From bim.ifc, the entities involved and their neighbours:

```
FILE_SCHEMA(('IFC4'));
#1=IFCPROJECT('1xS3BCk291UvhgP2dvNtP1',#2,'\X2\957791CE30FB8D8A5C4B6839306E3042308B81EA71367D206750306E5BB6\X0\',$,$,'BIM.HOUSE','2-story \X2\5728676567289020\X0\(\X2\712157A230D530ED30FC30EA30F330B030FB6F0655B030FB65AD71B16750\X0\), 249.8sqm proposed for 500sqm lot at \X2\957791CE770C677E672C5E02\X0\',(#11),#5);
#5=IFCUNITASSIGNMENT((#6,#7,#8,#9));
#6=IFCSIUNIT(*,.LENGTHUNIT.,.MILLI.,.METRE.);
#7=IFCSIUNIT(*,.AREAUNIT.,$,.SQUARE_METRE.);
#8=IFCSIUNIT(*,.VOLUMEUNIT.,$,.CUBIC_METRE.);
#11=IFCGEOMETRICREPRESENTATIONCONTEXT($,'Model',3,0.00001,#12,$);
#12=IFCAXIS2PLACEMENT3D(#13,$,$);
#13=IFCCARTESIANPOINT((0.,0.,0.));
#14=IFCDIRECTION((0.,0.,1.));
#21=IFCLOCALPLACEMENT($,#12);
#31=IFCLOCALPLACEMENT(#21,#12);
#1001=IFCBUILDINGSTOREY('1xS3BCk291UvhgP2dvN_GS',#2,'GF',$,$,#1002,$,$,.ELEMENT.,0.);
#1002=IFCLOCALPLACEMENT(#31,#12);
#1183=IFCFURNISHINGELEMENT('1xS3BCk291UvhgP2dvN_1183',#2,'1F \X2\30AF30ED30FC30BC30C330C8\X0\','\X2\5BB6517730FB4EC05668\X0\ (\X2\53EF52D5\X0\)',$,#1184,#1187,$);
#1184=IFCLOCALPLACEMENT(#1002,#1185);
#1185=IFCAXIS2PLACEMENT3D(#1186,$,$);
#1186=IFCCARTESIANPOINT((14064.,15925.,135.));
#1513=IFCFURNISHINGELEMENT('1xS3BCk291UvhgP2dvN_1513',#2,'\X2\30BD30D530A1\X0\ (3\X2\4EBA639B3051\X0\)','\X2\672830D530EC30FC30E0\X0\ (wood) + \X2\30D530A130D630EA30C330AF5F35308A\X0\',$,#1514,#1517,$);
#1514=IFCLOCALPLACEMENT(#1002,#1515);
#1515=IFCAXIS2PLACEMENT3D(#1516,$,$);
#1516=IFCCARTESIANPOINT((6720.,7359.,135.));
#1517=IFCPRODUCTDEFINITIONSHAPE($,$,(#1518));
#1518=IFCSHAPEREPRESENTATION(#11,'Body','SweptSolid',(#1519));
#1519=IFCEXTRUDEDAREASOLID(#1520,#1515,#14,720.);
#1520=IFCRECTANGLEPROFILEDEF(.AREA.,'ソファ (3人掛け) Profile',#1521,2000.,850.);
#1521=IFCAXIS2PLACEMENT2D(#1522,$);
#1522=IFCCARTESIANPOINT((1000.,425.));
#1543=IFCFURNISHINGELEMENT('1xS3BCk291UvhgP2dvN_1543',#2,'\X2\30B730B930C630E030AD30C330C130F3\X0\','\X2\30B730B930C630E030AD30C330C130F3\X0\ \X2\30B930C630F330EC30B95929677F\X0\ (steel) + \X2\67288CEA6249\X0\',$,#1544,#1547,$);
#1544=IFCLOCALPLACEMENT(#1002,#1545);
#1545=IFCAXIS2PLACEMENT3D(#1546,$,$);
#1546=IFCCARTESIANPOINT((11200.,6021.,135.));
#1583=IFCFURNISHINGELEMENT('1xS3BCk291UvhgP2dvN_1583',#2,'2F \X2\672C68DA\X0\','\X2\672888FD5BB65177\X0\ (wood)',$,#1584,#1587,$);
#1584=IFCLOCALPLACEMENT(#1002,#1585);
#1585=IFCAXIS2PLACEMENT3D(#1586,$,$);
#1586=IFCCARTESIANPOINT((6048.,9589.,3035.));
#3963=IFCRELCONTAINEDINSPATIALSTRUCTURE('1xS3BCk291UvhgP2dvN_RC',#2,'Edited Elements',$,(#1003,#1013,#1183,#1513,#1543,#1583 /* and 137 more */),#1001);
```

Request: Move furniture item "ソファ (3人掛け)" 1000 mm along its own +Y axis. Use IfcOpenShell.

```python
import ifcopenshell
import ifcopenshell.api.geometry
import ifcopenshell.util.placement
import ifcopenshell.util.unit

model = ifcopenshell.open("bim.ifc")
unit_scale = ifcopenshell.util.unit.calculate_unit_scale(model)

item = model.by_id(1513)
matrix = ifcopenshell.util.placement.get_local_placement(item.ObjectPlacement)
matrix[:3, 3] += matrix[:3, 1] * 1 / unit_scale
ifcopenshell.api.geometry.edit_object_placement(model, product=item, matrix=matrix, is_si=False)

print(ifcopenshell.util.placement.get_local_placement(item.ObjectPlacement).round(3) + 0.0)

model.write("bim_updated.ifc")
```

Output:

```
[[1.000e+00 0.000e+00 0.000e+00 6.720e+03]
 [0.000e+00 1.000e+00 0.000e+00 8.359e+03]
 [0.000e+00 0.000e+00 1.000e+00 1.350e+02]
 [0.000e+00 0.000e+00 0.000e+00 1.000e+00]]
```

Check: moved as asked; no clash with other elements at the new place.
